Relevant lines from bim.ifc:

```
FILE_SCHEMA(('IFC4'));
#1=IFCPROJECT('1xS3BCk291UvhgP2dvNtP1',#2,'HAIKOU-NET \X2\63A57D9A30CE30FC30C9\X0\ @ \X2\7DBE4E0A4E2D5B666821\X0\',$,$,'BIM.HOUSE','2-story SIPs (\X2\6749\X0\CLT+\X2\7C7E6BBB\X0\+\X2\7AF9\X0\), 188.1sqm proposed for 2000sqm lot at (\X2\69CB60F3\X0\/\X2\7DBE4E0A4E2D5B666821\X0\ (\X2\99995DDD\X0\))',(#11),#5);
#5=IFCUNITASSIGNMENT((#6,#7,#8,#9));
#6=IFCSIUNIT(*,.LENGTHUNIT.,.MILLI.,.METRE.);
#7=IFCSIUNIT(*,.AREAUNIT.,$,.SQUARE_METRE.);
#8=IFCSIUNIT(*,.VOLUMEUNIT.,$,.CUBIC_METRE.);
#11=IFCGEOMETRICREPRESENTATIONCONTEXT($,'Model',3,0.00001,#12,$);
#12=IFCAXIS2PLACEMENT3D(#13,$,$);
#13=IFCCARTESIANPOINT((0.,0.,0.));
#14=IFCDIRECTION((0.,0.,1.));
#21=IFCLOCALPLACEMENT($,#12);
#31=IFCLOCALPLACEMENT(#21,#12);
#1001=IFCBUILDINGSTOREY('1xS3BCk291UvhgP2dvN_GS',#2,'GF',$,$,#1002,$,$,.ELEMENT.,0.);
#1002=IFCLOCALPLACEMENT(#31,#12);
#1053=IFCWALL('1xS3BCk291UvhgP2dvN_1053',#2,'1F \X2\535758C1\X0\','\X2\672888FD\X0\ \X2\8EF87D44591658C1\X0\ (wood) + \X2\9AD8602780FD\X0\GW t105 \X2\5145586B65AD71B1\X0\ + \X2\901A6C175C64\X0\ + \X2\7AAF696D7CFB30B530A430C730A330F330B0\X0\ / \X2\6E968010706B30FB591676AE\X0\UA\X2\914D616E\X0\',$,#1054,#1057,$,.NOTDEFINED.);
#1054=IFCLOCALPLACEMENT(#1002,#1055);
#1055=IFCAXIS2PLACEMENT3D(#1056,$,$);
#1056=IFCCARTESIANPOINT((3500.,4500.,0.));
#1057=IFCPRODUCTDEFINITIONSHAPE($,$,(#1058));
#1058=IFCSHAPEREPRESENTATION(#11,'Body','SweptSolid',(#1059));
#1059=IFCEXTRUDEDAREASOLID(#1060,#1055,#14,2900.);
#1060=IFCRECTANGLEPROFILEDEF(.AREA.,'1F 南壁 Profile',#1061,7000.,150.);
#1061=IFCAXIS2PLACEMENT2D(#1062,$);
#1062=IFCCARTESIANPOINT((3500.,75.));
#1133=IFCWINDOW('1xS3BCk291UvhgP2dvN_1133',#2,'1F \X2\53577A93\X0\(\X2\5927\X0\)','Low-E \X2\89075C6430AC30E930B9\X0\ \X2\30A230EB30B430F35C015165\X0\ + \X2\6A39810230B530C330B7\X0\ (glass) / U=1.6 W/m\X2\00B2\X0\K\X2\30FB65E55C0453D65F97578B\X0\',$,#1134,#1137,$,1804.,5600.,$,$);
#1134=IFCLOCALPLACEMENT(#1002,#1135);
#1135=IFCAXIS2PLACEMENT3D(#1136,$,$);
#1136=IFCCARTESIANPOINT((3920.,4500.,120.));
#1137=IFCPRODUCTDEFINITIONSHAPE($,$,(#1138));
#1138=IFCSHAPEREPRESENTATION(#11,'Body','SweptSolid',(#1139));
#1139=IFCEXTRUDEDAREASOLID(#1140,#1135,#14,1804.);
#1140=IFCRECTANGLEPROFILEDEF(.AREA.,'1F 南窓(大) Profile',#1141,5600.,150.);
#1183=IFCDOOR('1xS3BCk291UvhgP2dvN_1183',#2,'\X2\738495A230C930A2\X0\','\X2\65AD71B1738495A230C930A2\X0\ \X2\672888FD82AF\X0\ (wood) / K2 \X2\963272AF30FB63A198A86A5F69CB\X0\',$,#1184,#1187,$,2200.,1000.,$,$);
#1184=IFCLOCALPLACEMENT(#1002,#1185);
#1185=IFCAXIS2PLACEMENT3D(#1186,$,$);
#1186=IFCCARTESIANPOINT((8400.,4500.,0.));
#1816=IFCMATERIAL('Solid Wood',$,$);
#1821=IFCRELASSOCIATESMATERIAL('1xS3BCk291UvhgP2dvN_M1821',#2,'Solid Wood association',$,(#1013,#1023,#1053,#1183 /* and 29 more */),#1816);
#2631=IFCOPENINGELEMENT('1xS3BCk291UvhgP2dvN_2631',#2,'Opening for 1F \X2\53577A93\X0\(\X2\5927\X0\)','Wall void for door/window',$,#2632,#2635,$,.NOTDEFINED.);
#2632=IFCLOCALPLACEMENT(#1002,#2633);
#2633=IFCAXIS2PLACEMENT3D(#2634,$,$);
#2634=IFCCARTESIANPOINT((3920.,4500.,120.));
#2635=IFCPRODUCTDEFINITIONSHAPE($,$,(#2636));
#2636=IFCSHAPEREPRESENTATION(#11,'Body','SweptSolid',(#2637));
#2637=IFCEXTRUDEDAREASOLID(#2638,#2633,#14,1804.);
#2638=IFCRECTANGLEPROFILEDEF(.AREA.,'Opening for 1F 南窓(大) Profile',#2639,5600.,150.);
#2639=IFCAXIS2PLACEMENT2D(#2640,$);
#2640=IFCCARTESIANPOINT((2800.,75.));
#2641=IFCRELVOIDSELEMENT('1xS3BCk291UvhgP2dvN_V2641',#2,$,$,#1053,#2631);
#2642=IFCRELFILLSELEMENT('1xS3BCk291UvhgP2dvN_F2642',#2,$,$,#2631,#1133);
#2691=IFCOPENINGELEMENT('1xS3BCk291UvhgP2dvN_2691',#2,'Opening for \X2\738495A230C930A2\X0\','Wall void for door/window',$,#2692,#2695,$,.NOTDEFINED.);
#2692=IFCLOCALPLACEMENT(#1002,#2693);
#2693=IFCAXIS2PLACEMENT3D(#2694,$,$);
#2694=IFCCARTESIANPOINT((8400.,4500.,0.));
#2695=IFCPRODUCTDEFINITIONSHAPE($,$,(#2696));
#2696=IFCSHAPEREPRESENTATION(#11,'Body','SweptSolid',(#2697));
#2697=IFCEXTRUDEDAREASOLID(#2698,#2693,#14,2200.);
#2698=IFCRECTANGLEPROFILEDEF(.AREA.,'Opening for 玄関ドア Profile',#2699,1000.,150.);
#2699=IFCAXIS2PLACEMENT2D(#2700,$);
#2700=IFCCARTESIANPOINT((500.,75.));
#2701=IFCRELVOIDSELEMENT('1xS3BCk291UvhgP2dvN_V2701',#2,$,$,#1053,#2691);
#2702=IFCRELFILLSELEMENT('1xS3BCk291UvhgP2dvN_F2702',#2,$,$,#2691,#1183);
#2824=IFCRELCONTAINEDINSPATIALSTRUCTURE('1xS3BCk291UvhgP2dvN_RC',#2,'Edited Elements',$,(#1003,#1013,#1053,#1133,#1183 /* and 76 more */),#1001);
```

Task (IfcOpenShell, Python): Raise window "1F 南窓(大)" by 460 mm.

```python
import numpy as np
import ifcopenshell
import ifcopenshell.api.geometry
import ifcopenshell.util.placement
import ifcopenshell.util.unit

model = ifcopenshell.open("bim.ifc")
unit_scale = ifcopenshell.util.unit.calculate_unit_scale(model)

window = model.by_id(1133)
opening = window.FillsVoids[0].RelatingOpeningElement
dz = 0.46 / unit_scale

shift = np.array([0.0, 0.0, dz])
# The window is not placed relative to its opening, so move both.
for product in (opening, window):
    matrix = ifcopenshell.util.placement.get_local_placement(product.ObjectPlacement)
    matrix[:3, 3] += shift
    ifcopenshell.api.geometry.edit_object_placement(model, product=product, matrix=matrix, is_si=False)

print(f"moved by {dz * unit_scale:+.3f} m")

model.write("bim-out.ifc")
```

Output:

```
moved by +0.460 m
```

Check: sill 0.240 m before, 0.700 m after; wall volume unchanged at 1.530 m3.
